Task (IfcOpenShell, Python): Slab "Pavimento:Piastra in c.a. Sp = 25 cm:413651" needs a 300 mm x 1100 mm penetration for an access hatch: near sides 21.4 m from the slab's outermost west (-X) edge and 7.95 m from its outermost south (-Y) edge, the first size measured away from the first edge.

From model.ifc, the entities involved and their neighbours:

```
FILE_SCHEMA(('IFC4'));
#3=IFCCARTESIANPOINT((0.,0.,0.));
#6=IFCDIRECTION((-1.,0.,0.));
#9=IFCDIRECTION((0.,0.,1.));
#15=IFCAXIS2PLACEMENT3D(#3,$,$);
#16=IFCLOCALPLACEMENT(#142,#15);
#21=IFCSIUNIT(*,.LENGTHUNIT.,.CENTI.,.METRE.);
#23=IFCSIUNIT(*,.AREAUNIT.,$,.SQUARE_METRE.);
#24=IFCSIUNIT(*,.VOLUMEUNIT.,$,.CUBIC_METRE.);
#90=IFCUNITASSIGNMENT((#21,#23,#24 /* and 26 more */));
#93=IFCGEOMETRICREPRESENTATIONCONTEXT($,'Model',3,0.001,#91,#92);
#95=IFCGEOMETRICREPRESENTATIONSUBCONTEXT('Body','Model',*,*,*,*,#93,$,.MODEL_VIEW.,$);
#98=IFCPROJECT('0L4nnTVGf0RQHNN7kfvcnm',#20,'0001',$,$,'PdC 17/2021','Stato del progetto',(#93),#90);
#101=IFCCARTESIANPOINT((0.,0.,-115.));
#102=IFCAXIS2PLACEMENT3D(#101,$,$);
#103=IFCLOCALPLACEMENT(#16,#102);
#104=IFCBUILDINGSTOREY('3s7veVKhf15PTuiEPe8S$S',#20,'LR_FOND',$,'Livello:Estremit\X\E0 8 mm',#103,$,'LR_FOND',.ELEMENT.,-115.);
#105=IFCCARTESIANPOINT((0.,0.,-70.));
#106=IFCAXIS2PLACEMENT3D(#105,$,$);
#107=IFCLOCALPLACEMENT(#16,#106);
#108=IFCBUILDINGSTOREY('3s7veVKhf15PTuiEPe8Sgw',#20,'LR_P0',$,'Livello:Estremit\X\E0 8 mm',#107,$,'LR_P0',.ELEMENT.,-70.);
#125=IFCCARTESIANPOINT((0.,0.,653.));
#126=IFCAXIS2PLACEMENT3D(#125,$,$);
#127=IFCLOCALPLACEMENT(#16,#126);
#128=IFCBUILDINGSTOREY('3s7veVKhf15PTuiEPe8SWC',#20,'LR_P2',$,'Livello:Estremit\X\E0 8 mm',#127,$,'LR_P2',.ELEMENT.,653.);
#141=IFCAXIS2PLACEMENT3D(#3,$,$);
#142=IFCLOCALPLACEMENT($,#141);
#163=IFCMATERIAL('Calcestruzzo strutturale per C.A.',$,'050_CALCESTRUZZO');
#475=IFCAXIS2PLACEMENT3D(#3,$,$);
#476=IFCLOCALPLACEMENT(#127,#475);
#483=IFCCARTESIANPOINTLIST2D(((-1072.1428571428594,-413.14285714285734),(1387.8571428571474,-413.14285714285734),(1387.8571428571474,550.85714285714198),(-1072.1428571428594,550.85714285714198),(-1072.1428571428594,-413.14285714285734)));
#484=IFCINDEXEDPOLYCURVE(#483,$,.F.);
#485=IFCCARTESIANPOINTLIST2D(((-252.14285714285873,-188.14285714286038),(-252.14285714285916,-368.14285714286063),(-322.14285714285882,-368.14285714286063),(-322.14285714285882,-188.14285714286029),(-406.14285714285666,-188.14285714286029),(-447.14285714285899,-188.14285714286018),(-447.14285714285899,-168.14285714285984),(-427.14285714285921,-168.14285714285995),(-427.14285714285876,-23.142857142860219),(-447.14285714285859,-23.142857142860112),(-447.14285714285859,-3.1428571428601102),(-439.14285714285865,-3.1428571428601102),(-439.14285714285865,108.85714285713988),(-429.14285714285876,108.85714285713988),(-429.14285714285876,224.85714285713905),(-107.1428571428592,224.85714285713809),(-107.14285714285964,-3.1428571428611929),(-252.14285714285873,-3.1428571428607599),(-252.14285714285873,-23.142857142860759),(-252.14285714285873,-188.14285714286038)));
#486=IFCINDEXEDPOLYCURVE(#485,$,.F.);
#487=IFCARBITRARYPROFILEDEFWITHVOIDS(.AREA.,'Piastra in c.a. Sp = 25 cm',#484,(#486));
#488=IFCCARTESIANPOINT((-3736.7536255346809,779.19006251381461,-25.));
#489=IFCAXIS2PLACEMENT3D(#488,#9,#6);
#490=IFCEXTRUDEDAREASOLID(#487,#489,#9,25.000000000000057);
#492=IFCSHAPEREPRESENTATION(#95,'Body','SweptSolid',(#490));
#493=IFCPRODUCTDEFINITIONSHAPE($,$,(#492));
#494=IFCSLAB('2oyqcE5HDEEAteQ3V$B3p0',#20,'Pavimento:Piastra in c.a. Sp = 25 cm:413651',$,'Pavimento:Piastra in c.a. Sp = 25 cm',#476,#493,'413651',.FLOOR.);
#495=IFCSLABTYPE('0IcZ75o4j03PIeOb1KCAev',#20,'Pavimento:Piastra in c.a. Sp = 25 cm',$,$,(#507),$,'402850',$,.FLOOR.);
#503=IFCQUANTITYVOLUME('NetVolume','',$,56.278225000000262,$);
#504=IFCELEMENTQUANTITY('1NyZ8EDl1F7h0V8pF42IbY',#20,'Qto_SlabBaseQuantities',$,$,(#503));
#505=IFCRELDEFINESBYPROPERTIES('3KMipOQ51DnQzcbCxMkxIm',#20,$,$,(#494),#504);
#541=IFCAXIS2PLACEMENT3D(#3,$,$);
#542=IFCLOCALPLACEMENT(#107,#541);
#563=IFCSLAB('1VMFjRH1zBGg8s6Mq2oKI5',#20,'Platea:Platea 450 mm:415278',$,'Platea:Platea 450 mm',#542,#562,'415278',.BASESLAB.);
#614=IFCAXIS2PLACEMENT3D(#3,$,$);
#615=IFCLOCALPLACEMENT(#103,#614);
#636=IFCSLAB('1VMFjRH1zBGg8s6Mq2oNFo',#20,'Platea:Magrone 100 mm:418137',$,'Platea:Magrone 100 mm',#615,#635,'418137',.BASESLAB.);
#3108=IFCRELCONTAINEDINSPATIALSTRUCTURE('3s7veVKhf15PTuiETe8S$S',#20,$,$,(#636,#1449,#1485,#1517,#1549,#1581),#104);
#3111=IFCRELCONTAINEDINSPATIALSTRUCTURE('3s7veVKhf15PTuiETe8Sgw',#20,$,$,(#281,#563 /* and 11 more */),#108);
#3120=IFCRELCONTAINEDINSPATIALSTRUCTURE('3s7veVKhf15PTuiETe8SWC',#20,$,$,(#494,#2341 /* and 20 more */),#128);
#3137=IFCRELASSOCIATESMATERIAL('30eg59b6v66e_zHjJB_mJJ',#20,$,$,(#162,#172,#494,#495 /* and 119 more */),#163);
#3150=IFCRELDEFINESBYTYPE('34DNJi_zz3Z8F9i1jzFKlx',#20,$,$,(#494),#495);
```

```python
import numpy as np
import ifcopenshell
import ifcopenshell.api.feature
import ifcopenshell.api.geometry
import ifcopenshell.api.pset
import ifcopenshell.api.root
import ifcopenshell.geom
import ifcopenshell.util.element
import ifcopenshell.util.placement
import ifcopenshell.util.representation
import ifcopenshell.util.shape
import ifcopenshell.util.unit

model = ifcopenshell.open("model.ifc")
unit_scale = ifcopenshell.util.unit.calculate_unit_scale(model)
volume_scale = ifcopenshell.util.unit.calculate_unit_scale(model, "VOLUMEUNIT")
settings = ifcopenshell.geom.settings()


def volume(element):
    """Net volume in cubic metres, openings subtracted."""
    shape = ifcopenshell.geom.create_shape(settings, element)
    return ifcopenshell.util.shape.get_volume(shape.geometry)


slab = model.by_guid("2oyqcE5HDEEAteQ3V$B3p0")
before = volume(slab)

# Extent in the slab's own axes, in metres. The edges named are its -X and -Y sides.
slab_shape = ifcopenshell.geom.create_shape(settings, slab)
vertices = ifcopenshell.util.shape.get_vertices(slab_shape.geometry)
x_min, y_min, bottom = vertices.min(axis=0)
top = vertices[:, 2].max()

opening = ifcopenshell.api.root.create_entity(model, ifc_class="IfcOpeningElement", name="Access hatch opening", predefined_type="OPENING")
context = ifcopenshell.util.representation.get_context(model, "Model", "Body", "MODEL_VIEW")
width, depth = 0.3, 1.1
outline = [(0.0, 0.0), (width, 0.0), (width, depth), (0.0, depth), (0.0, 0.0)]
# Overshoot both faces by 50 mm so the cut is clean.
shape = ifcopenshell.api.geometry.add_slab_representation(
    model, context=context, depth=top - bottom + 0.1, polyline=outline
)
ifcopenshell.api.geometry.assign_representation(model, product=opening, representation=shape)

matrix = ifcopenshell.util.placement.get_local_placement(slab.ObjectPlacement)
matrix[:, 3] = matrix @ np.append(np.array([x_min + 21.4, y_min + 7.95, bottom - 0.05]) / unit_scale, 1.0)
ifcopenshell.api.geometry.edit_object_placement(model, product=opening, matrix=matrix, is_si=False)
ifcopenshell.api.feature.add_feature(model, feature=opening, element=slab)

after = volume(slab)

# Update the slab's stored quantities.
qto = model.by_id(ifcopenshell.util.element.get_pset(slab, "Qto_SlabBaseQuantities", should_inherit=False)["id"])
ifcopenshell.api.pset.edit_qto(model, qto=qto, properties={"NetVolume": after / volume_scale})

print(f"slab volume {before:.3f} -> {after:.3f} m3")

model.write("model_edited.ifc")
```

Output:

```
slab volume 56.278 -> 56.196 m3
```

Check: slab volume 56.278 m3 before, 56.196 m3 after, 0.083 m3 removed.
